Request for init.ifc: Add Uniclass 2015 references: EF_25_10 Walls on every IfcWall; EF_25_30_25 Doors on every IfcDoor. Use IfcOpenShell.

First a look at what the model holds.

```python
import ifcopenshell

model = ifcopenshell.open("init.ifc")
print(model.schema)
print("classifications:", [c.Name for c in model.by_type("IfcClassification")])
for ifc_class in ("IfcDoor", "IfcRoof", "IfcStair", "IfcWall", "IfcWindow"):
    print(ifc_class, len(model.by_type(ifc_class)))
```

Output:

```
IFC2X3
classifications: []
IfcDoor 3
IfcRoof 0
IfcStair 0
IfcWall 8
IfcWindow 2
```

```python
import ifcopenshell
import ifcopenshell.api.classification

model = ifcopenshell.open("init.ifc")

# IFC2X3 requires Source and Edition and has no link from the project to the system.
system = model.create_entity("IfcClassification", Source="NBS", Edition="2015", Name="Uniclass 2015")

codes = {
    "IfcWall": ("EF_25_10", "Walls"),
    "IfcDoor": ("EF_25_30_25", "Doors"),
}
for ifc_class, (code, name) in codes.items():
    products = model.by_type(ifc_class)
    ifcopenshell.api.classification.add_reference(
        model, products=products, classification=system, identification=code, name=name
    )
    print(code, len(products))

model.write("init-out.ifc")
```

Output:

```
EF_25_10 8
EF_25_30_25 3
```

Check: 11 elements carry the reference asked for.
